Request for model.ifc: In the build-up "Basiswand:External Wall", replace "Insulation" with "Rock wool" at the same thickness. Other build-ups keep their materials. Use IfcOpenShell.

First a look at what the model holds.

```python
import ifcopenshell
import ifcopenshell.util.element

model = ifcopenshell.open("model.ifc")
print(model.schema)
for layer_set in model.by_type("IfcMaterialLayerSet"):
    if layer_set.LayerSetName == "Basiswand:External Wall":
        for layer in layer_set.MaterialLayers:
            print(layer.id(), layer.Material and layer.Material.Name, layer.LayerThickness, sep=" | ")
        print(len(ifcopenshell.util.element.get_elements_by_material(model, layer_set)), "elements and types use it")
print(sorted(m.Name for m in model.by_type("IfcMaterial") if m.Name)[:60])
```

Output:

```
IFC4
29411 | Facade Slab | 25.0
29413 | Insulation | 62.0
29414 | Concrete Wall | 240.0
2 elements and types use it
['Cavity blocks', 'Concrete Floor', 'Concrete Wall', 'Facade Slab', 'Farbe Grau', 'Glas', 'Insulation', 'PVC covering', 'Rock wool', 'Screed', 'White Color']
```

```python
import ifcopenshell
import ifcopenshell.api.material

model = ifcopenshell.open("model.ifc")

layer_set = next(s for s in model.by_type("IfcMaterialLayerSet") if s.LayerSetName == "Basiswand:External Wall")
layer = next(l for l in layer_set.MaterialLayers if l.Material and l.Material.Name == "Insulation")
material = next(m for m in model.by_type("IfcMaterial") if m.Name == "Rock wool")

# Point this one layer at the other material; renaming the old one would change it everywhere.
ifcopenshell.api.material.edit_layer(model, layer=layer, attributes={}, material=material)

print([l.Material.Name if l.Material else None for l in layer_set.MaterialLayers])

model.write("model_updated.ifc")
```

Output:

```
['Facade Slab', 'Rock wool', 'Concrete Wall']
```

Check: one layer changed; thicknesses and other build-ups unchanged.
